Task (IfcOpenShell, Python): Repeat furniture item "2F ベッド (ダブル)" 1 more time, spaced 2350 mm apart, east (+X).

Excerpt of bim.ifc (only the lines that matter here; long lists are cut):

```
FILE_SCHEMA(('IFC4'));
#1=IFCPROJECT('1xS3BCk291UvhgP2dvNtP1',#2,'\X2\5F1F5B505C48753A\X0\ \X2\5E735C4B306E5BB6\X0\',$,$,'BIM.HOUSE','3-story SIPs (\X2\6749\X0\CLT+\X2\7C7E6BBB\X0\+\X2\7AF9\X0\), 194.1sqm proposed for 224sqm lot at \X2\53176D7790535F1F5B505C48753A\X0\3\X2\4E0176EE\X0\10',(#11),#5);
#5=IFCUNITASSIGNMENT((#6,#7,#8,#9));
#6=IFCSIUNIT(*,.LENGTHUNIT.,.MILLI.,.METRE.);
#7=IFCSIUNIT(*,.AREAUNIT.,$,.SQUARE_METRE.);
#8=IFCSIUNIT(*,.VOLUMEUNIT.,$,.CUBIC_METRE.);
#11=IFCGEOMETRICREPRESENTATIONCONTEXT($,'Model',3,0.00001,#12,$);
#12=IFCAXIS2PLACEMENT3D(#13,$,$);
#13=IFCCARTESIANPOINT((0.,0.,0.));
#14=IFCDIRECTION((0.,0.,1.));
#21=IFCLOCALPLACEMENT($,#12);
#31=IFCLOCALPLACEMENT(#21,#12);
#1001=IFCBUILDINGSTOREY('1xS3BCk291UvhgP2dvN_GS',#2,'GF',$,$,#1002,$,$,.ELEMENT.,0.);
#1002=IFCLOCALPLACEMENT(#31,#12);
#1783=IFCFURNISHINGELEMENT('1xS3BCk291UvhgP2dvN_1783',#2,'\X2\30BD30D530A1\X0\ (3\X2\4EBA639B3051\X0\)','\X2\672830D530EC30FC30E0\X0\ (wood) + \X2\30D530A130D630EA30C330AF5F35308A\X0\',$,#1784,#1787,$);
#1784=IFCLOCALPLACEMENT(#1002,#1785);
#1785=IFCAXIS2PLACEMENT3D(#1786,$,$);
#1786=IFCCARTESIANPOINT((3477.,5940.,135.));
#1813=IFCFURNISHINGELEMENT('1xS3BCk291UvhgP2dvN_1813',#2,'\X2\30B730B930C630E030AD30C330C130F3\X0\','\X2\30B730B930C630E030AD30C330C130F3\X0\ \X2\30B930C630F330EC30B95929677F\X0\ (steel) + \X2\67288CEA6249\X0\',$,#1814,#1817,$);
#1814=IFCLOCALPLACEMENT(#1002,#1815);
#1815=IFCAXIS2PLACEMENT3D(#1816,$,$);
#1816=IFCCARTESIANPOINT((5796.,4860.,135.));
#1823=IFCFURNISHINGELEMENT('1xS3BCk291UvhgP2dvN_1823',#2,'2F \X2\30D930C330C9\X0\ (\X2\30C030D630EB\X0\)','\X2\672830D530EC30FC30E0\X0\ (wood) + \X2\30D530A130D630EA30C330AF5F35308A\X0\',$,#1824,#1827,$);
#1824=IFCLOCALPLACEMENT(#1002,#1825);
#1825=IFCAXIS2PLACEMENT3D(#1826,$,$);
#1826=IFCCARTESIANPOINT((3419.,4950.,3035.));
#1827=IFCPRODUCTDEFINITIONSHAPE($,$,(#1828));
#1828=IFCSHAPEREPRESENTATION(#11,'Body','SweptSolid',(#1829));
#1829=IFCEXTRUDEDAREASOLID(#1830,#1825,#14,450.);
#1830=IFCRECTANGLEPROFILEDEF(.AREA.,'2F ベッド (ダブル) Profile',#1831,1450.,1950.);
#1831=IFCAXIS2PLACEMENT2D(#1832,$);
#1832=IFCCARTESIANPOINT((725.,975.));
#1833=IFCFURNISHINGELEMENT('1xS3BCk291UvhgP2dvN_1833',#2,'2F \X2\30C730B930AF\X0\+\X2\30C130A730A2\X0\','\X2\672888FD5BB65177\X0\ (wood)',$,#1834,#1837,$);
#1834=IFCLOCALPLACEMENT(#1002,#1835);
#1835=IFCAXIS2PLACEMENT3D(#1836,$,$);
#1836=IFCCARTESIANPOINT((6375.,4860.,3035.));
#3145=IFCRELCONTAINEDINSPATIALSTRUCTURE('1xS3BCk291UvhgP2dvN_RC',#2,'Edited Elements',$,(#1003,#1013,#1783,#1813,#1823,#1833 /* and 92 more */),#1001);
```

```python
import numpy as np
import ifcopenshell
import ifcopenshell.api.geometry
import ifcopenshell.api.root
import ifcopenshell.util.element
import ifcopenshell.util.placement
import ifcopenshell.util.unit

model = ifcopenshell.open("bim.ifc")
unit_scale = ifcopenshell.util.unit.calculate_unit_scale(model)


def reuse_history(source, copy):
    """copy_class also copies each property set's owner history, people and application; keep the originals."""
    for rel in copy.IsDefinedBy:
        if rel.is_a("IfcRelDefinesByProperties") and (history := rel.RelatingPropertyDefinition.OwnerHistory):
            rel.RelatingPropertyDefinition.OwnerHistory = source.OwnerHistory
            ifcopenshell.util.element.remove_deep2(model, history)


source = model.by_guid("1xS3BCk291UvhgP2dvN_1823")
base = ifcopenshell.util.placement.get_local_placement(source.ObjectPlacement)
step = np.array([1.0, 0.0, 0.0]) * 2.35 / unit_scale

for i in range(1, 2):
    copy = ifcopenshell.api.root.copy_class(model, product=source)
    copy.Representation = ifcopenshell.util.element.copy_deep(
        model, source.Representation, exclude=["IfcGeometricRepresentationContext", "IfcRepresentationMap"]
    )
    reuse_history(source, copy)
    matrix = base.copy()
    matrix[:3, 3] += i * step
    print("added at", matrix[:3, 3].round(3) + 0.0)
    ifcopenshell.api.geometry.edit_object_placement(model, product=copy, matrix=matrix, is_si=False)

model.write("bim_edited.ifc")
```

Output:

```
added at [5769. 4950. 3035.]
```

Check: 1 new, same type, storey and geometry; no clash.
